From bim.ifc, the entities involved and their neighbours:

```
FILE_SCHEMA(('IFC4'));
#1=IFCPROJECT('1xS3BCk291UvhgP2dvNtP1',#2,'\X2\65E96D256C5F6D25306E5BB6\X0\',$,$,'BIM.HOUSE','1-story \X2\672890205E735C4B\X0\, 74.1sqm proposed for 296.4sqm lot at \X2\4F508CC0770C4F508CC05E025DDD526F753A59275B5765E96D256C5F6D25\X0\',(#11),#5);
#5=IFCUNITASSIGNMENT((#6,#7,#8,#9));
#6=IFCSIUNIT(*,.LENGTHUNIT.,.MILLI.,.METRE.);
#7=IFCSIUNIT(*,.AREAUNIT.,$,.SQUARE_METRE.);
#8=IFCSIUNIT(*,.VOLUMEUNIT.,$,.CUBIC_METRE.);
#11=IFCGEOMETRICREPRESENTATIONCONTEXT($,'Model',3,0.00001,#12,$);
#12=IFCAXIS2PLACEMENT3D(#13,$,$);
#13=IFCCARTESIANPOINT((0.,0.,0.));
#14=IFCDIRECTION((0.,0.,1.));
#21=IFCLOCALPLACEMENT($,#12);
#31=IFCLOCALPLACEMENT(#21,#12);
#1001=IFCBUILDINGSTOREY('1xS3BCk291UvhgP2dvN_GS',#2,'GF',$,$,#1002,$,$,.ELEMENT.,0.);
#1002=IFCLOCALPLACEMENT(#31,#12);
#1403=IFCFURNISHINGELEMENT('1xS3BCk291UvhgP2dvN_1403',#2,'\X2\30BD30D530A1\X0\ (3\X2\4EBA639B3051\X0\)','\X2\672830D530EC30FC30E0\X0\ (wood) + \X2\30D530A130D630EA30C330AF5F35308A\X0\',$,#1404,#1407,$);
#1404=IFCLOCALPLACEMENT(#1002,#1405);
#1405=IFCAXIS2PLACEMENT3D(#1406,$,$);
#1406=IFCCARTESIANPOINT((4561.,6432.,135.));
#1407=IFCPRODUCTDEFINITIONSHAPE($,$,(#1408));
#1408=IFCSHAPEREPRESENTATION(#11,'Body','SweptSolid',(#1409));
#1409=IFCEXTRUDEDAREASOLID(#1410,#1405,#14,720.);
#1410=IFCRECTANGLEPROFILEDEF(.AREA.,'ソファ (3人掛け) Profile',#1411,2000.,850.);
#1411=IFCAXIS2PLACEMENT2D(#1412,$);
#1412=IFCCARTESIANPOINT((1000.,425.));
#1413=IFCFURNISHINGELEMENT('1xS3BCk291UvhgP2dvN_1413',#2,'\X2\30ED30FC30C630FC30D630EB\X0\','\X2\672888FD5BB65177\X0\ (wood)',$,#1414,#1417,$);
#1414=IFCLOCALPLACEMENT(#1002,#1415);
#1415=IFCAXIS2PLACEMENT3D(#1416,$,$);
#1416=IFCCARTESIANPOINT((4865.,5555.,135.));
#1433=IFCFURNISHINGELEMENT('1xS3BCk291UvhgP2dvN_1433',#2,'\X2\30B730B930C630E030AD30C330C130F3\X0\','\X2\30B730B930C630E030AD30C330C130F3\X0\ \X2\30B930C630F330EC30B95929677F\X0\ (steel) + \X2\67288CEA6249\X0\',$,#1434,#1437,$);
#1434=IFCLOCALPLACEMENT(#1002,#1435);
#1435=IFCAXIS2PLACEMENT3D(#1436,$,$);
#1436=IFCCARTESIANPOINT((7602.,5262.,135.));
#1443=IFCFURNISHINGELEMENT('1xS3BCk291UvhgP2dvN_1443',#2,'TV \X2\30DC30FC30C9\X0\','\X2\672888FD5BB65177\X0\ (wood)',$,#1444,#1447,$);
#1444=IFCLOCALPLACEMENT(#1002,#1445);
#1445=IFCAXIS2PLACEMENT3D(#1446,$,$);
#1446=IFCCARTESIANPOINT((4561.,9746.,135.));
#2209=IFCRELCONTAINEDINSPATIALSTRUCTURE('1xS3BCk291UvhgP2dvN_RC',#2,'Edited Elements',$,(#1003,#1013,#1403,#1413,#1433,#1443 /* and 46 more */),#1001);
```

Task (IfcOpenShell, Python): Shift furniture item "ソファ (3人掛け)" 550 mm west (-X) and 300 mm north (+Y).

```python
import ifcopenshell
import ifcopenshell.api.geometry
import ifcopenshell.util.placement

model = ifcopenshell.open("bim.ifc")

item = model.by_id(1403)
matrix = ifcopenshell.util.placement.get_local_placement(item.ObjectPlacement)
matrix[0, 3] -= 550.0
matrix[1, 3] += 300.0
ifcopenshell.api.geometry.edit_object_placement(model, product=item, matrix=matrix, is_si=False)

print(ifcopenshell.util.placement.get_local_placement(item.ObjectPlacement).round(3) + 0.0)

model.write("bim-out.ifc")
```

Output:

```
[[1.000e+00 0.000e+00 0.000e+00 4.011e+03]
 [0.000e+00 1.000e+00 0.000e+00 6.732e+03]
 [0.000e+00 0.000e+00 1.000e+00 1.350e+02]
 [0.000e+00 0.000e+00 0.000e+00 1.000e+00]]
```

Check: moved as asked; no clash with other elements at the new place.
